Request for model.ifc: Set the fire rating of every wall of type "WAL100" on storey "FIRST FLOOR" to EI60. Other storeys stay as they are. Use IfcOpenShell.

First a look at what the model holds.

```python
import ifcopenshell
import ifcopenshell.util.element

model = ifcopenshell.open("model.ifc")
print(model.schema)
storey = next(s for s in model.by_type("IfcBuildingStorey") if s.Name == "FIRST FLOOR")
walls = [e for e in ifcopenshell.util.element.get_decomposition(storey) if e.is_a("IfcWall")]
seen = {}
for e in walls:
    element_type = ifcopenshell.util.element.get_type(e)
    key = (element_type.Name if element_type != e and element_type else None, ifcopenshell.util.element.get_pset(e, "Pset_WallCommon", "FireRating"))
    seen[key] = seen.get(key, 0) + 1
for (name, value), count in sorted(seen.items(), key=str):
    print(count, "x", name, "|", value)
```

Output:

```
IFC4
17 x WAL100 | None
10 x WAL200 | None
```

```python
import ifcopenshell
import ifcopenshell.api.pset
import ifcopenshell.util.element

model = ifcopenshell.open("model.ifc")

storey = next(s for s in model.by_type("IfcBuildingStorey") if s.Name == "FIRST FLOOR")
walls = [e for e in ifcopenshell.util.element.get_decomposition(storey) if e.is_a("IfcWall")]

count = 0
for e in walls:
    element_type = ifcopenshell.util.element.get_type(e)
    if element_type in (None, e) or element_type.Name != "WAL100":
        continue
    # add_pset returns the element's existing set when there is one.
    pset = ifcopenshell.api.pset.add_pset(model, product=e, name="Pset_WallCommon")
    ifcopenshell.api.pset.edit_pset(model, pset=pset, properties={"FireRating": "EI60"})
    count += 1

print(count, "walls updated")

model.write("model_edited.ifc")
```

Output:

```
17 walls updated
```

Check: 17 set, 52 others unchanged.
